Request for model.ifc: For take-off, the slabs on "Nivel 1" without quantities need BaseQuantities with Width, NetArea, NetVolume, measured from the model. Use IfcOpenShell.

First a look at what the model holds.

```python
import ifcopenshell
import ifcopenshell.util.element
import ifcopenshell.util.unit

model = ifcopenshell.open("model.ifc")
print(model.schema)
for unit_type in ("LENGTHUNIT", "AREAUNIT", "VOLUMEUNIT"):
    print(unit_type, ifcopenshell.util.unit.calculate_unit_scale(model, unit_type))
storey = next(s for s in model.by_type("IfcBuildingStorey") if s.Name == "Nivel 1")
slabs = [e for e in ifcopenshell.util.element.get_decomposition(storey) if e.is_a("IfcSlab")]
for e in sorted(slabs, key=lambda e: e.id()):
    print(e.id(), e.is_a(), e.Name, list(ifcopenshell.util.element.get_psets(e, qtos_only=True)), sep=" | ")
```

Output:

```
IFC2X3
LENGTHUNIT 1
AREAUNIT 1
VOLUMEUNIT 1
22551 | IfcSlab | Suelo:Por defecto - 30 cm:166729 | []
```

```python
import ifcopenshell
import ifcopenshell.api.pset
import ifcopenshell.geom
import ifcopenshell.util.element
import ifcopenshell.util.shape
import ifcopenshell.util.unit

model = ifcopenshell.open("model.ifc")
unit_scale = ifcopenshell.util.unit.calculate_unit_scale(model)
area_scale = ifcopenshell.util.unit.calculate_unit_scale(model, "AREAUNIT")
volume_scale = ifcopenshell.util.unit.calculate_unit_scale(model, "VOLUMEUNIT")
settings = ifcopenshell.geom.settings()

storey = next(s for s in model.by_type("IfcBuildingStorey") if s.Name == "Nivel 1")
slabs = [e for e in ifcopenshell.util.element.get_decomposition(storey) if e.is_a("IfcSlab")]

for e in sorted(slabs, key=lambda e: e.id()):
    if ifcopenshell.util.element.get_psets(e, qtos_only=True, should_inherit=False):
        continue
    # Geometry comes back in metres, in the element's own axes.
    shape = ifcopenshell.geom.create_shape(settings, e)
    values = {
        "Width": ifcopenshell.util.shape.get_z(shape.geometry) / unit_scale,
        "NetArea": ifcopenshell.util.shape.get_footprint_area(shape.geometry) / area_scale,
        "NetVolume": ifcopenshell.util.shape.get_volume(shape.geometry) / volume_scale,
    }
    qto = ifcopenshell.api.pset.add_qto(model, product=e, name="BaseQuantities")
    ifcopenshell.api.pset.edit_qto(model, qto=qto, properties=values)
    print(e.id(), {k: round(v, 3) for k, v in values.items()})

model.write("model_edited.ifc")
```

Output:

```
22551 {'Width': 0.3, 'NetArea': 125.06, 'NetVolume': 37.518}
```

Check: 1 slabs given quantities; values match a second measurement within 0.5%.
